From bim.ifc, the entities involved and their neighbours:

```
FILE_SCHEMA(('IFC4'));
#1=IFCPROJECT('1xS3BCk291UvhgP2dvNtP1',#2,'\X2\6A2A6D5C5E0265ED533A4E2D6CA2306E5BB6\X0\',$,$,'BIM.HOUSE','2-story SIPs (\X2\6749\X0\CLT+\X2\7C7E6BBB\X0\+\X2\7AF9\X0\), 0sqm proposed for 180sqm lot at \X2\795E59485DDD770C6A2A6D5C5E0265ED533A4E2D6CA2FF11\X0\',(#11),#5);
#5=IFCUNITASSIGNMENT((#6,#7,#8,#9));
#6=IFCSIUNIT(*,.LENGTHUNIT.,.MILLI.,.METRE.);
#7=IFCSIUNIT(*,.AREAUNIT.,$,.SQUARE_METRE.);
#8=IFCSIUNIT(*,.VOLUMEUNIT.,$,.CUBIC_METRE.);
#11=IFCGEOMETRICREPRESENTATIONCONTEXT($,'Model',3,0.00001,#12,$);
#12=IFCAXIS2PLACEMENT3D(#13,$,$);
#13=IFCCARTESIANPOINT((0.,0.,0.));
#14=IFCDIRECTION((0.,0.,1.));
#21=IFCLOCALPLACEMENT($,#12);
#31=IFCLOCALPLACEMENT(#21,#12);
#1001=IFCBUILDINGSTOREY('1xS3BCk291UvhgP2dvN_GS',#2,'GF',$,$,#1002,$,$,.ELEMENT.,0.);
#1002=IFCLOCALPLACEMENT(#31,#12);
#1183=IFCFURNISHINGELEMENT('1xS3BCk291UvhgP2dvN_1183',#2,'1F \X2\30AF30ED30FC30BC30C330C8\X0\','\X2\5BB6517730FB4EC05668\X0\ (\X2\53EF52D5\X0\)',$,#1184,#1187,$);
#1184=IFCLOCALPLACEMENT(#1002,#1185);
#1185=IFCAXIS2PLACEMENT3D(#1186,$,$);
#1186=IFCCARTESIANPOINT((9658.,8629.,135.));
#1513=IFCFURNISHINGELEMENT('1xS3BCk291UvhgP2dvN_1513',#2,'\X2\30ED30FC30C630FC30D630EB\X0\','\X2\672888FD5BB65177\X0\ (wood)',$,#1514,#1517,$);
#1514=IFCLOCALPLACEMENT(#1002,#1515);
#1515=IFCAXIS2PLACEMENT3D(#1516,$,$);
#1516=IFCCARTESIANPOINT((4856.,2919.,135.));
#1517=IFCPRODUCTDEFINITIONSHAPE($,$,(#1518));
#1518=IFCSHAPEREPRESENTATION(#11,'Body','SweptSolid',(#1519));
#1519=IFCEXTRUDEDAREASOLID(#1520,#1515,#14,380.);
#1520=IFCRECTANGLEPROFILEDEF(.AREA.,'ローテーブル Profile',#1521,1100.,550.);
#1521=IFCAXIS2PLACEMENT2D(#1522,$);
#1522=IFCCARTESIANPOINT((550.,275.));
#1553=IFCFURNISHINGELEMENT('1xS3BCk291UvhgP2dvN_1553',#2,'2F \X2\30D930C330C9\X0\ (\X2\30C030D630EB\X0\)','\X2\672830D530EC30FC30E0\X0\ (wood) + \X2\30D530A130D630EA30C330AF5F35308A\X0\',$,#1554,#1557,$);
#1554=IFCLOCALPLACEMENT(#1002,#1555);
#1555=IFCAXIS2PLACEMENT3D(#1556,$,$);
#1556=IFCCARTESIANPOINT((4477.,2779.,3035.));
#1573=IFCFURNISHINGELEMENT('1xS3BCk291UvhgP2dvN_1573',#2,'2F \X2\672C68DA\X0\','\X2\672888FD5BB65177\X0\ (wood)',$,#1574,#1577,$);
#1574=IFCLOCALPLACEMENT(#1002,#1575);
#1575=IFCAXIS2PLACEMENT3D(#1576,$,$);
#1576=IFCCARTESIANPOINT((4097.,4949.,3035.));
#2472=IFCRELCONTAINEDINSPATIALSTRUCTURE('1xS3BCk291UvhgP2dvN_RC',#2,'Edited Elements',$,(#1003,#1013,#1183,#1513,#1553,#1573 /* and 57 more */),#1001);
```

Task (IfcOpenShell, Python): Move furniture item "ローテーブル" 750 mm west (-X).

```python
import ifcopenshell
import ifcopenshell.api.geometry
import ifcopenshell.util.placement
import ifcopenshell.util.unit

model = ifcopenshell.open("bim.ifc")
unit_scale = ifcopenshell.util.unit.calculate_unit_scale(model)

item = model.by_guid("1xS3BCk291UvhgP2dvN_1513")
matrix = ifcopenshell.util.placement.get_local_placement(item.ObjectPlacement)
matrix[0, 3] -= 0.75 / unit_scale
ifcopenshell.api.geometry.edit_object_placement(model, product=item, matrix=matrix, is_si=False)

print(ifcopenshell.util.placement.get_local_placement(item.ObjectPlacement).round(3) + 0.0)

model.write("bim_rev.ifc")
```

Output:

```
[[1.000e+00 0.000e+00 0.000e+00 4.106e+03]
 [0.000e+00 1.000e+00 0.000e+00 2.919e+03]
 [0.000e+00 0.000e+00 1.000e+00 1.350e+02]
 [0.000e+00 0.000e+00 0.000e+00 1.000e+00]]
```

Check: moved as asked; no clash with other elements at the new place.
